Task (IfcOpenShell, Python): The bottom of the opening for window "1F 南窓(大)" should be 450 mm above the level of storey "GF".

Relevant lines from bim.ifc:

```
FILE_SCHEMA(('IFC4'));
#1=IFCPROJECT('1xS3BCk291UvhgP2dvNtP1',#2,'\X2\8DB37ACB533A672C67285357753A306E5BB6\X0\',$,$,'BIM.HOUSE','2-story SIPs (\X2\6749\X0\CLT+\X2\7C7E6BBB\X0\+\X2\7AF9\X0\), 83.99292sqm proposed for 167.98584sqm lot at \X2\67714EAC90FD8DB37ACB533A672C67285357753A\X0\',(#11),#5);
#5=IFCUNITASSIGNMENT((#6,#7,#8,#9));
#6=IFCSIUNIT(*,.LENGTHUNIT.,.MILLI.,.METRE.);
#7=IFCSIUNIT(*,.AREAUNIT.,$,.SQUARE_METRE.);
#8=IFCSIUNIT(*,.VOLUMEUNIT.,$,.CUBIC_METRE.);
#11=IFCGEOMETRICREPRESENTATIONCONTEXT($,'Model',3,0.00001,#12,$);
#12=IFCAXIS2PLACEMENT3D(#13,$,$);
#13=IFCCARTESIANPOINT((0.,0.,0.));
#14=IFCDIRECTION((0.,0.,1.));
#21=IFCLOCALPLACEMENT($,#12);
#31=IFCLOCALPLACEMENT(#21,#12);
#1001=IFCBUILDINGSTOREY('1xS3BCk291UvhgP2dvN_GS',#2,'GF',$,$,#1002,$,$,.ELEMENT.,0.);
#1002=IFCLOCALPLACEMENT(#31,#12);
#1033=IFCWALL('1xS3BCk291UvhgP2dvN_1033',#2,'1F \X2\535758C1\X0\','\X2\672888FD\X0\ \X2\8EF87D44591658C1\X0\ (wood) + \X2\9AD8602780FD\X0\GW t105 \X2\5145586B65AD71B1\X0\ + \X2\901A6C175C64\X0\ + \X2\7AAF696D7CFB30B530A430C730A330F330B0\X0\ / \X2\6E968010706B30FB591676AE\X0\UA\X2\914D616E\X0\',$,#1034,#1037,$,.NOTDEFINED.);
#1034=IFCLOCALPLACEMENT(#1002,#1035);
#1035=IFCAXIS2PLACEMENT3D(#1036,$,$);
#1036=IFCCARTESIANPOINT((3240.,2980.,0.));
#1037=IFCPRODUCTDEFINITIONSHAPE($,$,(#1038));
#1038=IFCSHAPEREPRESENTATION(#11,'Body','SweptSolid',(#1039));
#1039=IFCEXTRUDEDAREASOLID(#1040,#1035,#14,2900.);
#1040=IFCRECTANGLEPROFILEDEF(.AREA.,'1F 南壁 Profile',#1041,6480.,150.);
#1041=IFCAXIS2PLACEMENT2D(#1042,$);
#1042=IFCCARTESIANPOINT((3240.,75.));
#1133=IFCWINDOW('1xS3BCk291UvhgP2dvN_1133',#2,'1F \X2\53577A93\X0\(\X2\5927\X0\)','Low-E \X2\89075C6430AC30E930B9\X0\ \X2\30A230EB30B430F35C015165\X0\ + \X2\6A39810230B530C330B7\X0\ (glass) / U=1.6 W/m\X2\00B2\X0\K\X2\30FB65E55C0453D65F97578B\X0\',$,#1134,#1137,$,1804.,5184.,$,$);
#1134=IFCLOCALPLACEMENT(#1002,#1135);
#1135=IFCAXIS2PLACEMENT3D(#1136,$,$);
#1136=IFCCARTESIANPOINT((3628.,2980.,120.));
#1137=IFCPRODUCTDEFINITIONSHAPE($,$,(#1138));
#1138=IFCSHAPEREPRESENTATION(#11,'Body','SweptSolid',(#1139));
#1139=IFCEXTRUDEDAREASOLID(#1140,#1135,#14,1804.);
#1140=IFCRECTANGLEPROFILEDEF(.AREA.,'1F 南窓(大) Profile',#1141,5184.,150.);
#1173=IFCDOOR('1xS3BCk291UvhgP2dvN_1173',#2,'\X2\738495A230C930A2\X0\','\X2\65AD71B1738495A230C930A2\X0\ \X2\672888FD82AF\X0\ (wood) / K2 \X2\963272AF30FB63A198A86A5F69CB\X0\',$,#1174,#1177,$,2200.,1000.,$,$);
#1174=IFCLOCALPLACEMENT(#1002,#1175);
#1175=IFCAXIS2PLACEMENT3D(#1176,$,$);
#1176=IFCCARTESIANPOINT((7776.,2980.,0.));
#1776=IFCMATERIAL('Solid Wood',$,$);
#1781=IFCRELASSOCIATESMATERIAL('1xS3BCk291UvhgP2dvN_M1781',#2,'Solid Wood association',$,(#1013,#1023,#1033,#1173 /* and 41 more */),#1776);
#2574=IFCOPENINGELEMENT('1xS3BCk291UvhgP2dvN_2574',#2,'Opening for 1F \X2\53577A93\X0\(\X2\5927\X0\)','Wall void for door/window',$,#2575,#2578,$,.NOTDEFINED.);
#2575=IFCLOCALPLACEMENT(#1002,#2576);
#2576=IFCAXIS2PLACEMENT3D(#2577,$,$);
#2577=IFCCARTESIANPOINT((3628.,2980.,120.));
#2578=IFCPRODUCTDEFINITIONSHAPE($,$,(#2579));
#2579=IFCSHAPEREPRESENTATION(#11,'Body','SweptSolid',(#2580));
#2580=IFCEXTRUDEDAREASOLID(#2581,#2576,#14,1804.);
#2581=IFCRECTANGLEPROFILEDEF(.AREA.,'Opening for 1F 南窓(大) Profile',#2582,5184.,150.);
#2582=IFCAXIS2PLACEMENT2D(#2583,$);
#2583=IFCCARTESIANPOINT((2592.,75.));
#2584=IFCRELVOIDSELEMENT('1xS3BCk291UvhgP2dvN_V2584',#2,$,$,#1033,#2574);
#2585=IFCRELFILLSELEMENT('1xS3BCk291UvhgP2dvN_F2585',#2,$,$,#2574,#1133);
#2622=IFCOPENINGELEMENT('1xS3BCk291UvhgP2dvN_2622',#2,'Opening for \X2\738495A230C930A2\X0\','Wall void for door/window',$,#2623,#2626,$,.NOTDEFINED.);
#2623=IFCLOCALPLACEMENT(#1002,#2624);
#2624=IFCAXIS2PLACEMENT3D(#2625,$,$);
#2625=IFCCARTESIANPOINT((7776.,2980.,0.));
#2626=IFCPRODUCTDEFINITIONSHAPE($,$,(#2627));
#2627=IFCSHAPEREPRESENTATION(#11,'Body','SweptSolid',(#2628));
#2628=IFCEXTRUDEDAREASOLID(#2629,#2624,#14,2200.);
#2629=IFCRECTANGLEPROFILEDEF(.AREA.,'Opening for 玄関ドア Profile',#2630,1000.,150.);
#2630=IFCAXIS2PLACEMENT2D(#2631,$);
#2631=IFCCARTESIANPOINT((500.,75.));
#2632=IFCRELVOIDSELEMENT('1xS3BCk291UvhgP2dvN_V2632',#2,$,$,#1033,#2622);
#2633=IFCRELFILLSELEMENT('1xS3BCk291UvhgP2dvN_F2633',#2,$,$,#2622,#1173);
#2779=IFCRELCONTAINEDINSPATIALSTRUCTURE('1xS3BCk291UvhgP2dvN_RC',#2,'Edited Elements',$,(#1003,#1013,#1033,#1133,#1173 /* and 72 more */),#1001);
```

```python
import numpy as np
import ifcopenshell
import ifcopenshell.api.geometry
import ifcopenshell.geom
import ifcopenshell.util.element
import ifcopenshell.util.placement
import ifcopenshell.util.shape
import ifcopenshell.util.unit

model = ifcopenshell.open("bim.ifc")
unit_scale = ifcopenshell.util.unit.calculate_unit_scale(model)

window = model.by_guid("1xS3BCk291UvhgP2dvN_1133")
opening = window.FillsVoids[0].RelatingOpeningElement
storey = ifcopenshell.util.element.get_container(window, ifc_class="IfcBuildingStorey")
level = ifcopenshell.util.placement.get_local_placement(storey.ObjectPlacement)[2, 3]

# The opening's origin need not be at the sill, so measure its lowest point.
shape = ifcopenshell.geom.create_shape(ifcopenshell.geom.settings(), opening)
bottom = ifcopenshell.util.shape.get_shape_bottom_elevation(shape, shape.geometry) / unit_scale
dz = level + 450.0 - bottom

shift = np.array([0.0, 0.0, dz])
# The window is not placed relative to its opening, so move both.
for product in (opening, window):
    matrix = ifcopenshell.util.placement.get_local_placement(product.ObjectPlacement)
    matrix[:3, 3] += shift
    ifcopenshell.api.geometry.edit_object_placement(model, product=product, matrix=matrix, is_si=False)

print(f"moved by {dz * unit_scale:+.3f} m")

model.write("bim_rev.ifc")
```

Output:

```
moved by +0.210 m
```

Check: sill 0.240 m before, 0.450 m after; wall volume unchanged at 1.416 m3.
